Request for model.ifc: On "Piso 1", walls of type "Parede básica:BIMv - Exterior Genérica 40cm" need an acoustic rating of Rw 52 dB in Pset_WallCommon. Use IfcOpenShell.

First a look at what the model holds.

```python
import ifcopenshell
import ifcopenshell.util.element

model = ifcopenshell.open("model.ifc")
print(model.schema)
storey = next(s for s in model.by_type("IfcBuildingStorey") if s.Name == "Piso 1")
walls = [e for e in ifcopenshell.util.element.get_decomposition(storey) if e.is_a("IfcWall")]
seen = {}
for e in walls:
    element_type = ifcopenshell.util.element.get_type(e)
    key = (element_type.Name if element_type != e and element_type else None, ifcopenshell.util.element.get_pset(e, "Pset_WallCommon", "AcousticRating"))
    seen[key] = seen.get(key, 0) + 1
for (name, value), count in sorted(seen.items(), key=str):
    print(count, "x", name, "|", value)
```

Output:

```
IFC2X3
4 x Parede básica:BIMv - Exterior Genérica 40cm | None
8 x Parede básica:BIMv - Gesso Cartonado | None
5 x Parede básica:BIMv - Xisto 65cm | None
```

```python
import ifcopenshell
import ifcopenshell.api.pset
import ifcopenshell.util.element

model = ifcopenshell.open("model.ifc")

storey = next(s for s in model.by_type("IfcBuildingStorey") if s.Name == "Piso 1")
walls = [e for e in ifcopenshell.util.element.get_decomposition(storey) if e.is_a("IfcWall")]

count = 0
for e in walls:
    element_type = ifcopenshell.util.element.get_type(e)
    if element_type in (None, e) or element_type.Name != "Parede básica:BIMv - Exterior Genérica 40cm":
        continue
    # add_pset returns the element's existing set when there is one.
    pset = ifcopenshell.api.pset.add_pset(model, product=e, name="Pset_WallCommon")
    ifcopenshell.api.pset.edit_pset(model, pset=pset, properties={"AcousticRating": "Rw 52 dB"})
    count += 1

print(count, "walls updated")

model.write("model_v2.ifc")
```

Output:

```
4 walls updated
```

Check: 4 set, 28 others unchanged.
